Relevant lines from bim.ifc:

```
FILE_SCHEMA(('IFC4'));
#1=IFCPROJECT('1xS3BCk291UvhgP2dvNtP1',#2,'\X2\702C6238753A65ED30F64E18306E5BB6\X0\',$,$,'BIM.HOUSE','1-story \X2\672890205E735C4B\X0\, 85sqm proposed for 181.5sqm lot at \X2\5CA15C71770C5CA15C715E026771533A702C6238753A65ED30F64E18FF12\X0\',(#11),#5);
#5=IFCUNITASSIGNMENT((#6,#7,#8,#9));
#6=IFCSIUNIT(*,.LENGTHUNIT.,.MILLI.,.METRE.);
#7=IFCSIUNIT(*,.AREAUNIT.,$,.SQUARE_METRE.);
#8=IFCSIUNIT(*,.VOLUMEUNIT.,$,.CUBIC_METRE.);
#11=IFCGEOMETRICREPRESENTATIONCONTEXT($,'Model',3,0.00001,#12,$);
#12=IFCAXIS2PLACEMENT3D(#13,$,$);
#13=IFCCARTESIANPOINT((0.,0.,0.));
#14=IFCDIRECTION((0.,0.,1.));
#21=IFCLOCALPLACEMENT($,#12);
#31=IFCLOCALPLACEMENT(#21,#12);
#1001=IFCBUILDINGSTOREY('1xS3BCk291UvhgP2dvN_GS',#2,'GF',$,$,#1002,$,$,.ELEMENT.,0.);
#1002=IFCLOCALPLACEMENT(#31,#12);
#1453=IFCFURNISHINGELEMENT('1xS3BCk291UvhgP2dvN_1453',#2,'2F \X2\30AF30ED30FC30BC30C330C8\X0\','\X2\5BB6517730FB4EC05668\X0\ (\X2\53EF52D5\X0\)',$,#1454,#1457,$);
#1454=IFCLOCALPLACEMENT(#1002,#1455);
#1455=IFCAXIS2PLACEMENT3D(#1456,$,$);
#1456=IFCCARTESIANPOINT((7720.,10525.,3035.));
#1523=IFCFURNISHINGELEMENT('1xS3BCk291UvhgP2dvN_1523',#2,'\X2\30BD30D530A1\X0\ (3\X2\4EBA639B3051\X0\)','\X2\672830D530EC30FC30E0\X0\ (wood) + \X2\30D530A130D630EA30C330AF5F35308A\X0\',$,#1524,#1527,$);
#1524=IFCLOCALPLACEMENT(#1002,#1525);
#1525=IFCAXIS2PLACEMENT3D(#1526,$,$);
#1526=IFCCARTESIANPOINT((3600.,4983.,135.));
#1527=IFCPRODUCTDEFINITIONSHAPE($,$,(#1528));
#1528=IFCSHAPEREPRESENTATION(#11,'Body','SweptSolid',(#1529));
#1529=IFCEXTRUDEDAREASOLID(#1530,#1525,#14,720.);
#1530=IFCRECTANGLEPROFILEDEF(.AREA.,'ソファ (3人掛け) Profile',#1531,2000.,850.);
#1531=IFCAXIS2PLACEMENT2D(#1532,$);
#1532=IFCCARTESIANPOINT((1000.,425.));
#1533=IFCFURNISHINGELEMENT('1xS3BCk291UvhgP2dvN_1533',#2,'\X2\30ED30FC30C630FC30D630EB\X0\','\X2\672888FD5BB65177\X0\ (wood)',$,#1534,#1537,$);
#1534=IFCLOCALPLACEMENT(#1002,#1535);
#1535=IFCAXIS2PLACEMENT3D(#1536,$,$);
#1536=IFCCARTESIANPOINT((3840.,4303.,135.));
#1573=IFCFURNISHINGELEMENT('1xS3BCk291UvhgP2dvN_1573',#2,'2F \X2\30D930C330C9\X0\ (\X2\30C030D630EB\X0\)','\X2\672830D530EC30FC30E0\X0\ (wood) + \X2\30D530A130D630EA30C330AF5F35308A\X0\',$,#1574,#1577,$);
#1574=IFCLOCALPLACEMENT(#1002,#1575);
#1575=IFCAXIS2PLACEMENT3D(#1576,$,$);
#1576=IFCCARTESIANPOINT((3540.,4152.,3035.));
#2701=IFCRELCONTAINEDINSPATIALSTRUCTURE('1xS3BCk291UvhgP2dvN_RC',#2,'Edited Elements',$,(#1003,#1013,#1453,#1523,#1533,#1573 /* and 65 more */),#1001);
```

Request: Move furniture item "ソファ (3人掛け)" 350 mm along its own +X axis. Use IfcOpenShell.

```python
import ifcopenshell
import ifcopenshell.api.geometry
import ifcopenshell.util.placement

model = ifcopenshell.open("bim.ifc")

item = model.by_id(1523)
matrix = ifcopenshell.util.placement.get_local_placement(item.ObjectPlacement)
matrix[:3, 3] += matrix[:3, 0] * 350.0
ifcopenshell.api.geometry.edit_object_placement(model, product=item, matrix=matrix, is_si=False)

print(ifcopenshell.util.placement.get_local_placement(item.ObjectPlacement).round(3) + 0.0)

model.write("bim_edited.ifc")
```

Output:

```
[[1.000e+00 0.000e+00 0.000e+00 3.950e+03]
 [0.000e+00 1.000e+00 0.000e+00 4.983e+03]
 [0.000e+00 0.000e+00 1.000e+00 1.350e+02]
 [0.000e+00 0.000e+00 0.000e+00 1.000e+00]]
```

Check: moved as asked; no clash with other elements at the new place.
